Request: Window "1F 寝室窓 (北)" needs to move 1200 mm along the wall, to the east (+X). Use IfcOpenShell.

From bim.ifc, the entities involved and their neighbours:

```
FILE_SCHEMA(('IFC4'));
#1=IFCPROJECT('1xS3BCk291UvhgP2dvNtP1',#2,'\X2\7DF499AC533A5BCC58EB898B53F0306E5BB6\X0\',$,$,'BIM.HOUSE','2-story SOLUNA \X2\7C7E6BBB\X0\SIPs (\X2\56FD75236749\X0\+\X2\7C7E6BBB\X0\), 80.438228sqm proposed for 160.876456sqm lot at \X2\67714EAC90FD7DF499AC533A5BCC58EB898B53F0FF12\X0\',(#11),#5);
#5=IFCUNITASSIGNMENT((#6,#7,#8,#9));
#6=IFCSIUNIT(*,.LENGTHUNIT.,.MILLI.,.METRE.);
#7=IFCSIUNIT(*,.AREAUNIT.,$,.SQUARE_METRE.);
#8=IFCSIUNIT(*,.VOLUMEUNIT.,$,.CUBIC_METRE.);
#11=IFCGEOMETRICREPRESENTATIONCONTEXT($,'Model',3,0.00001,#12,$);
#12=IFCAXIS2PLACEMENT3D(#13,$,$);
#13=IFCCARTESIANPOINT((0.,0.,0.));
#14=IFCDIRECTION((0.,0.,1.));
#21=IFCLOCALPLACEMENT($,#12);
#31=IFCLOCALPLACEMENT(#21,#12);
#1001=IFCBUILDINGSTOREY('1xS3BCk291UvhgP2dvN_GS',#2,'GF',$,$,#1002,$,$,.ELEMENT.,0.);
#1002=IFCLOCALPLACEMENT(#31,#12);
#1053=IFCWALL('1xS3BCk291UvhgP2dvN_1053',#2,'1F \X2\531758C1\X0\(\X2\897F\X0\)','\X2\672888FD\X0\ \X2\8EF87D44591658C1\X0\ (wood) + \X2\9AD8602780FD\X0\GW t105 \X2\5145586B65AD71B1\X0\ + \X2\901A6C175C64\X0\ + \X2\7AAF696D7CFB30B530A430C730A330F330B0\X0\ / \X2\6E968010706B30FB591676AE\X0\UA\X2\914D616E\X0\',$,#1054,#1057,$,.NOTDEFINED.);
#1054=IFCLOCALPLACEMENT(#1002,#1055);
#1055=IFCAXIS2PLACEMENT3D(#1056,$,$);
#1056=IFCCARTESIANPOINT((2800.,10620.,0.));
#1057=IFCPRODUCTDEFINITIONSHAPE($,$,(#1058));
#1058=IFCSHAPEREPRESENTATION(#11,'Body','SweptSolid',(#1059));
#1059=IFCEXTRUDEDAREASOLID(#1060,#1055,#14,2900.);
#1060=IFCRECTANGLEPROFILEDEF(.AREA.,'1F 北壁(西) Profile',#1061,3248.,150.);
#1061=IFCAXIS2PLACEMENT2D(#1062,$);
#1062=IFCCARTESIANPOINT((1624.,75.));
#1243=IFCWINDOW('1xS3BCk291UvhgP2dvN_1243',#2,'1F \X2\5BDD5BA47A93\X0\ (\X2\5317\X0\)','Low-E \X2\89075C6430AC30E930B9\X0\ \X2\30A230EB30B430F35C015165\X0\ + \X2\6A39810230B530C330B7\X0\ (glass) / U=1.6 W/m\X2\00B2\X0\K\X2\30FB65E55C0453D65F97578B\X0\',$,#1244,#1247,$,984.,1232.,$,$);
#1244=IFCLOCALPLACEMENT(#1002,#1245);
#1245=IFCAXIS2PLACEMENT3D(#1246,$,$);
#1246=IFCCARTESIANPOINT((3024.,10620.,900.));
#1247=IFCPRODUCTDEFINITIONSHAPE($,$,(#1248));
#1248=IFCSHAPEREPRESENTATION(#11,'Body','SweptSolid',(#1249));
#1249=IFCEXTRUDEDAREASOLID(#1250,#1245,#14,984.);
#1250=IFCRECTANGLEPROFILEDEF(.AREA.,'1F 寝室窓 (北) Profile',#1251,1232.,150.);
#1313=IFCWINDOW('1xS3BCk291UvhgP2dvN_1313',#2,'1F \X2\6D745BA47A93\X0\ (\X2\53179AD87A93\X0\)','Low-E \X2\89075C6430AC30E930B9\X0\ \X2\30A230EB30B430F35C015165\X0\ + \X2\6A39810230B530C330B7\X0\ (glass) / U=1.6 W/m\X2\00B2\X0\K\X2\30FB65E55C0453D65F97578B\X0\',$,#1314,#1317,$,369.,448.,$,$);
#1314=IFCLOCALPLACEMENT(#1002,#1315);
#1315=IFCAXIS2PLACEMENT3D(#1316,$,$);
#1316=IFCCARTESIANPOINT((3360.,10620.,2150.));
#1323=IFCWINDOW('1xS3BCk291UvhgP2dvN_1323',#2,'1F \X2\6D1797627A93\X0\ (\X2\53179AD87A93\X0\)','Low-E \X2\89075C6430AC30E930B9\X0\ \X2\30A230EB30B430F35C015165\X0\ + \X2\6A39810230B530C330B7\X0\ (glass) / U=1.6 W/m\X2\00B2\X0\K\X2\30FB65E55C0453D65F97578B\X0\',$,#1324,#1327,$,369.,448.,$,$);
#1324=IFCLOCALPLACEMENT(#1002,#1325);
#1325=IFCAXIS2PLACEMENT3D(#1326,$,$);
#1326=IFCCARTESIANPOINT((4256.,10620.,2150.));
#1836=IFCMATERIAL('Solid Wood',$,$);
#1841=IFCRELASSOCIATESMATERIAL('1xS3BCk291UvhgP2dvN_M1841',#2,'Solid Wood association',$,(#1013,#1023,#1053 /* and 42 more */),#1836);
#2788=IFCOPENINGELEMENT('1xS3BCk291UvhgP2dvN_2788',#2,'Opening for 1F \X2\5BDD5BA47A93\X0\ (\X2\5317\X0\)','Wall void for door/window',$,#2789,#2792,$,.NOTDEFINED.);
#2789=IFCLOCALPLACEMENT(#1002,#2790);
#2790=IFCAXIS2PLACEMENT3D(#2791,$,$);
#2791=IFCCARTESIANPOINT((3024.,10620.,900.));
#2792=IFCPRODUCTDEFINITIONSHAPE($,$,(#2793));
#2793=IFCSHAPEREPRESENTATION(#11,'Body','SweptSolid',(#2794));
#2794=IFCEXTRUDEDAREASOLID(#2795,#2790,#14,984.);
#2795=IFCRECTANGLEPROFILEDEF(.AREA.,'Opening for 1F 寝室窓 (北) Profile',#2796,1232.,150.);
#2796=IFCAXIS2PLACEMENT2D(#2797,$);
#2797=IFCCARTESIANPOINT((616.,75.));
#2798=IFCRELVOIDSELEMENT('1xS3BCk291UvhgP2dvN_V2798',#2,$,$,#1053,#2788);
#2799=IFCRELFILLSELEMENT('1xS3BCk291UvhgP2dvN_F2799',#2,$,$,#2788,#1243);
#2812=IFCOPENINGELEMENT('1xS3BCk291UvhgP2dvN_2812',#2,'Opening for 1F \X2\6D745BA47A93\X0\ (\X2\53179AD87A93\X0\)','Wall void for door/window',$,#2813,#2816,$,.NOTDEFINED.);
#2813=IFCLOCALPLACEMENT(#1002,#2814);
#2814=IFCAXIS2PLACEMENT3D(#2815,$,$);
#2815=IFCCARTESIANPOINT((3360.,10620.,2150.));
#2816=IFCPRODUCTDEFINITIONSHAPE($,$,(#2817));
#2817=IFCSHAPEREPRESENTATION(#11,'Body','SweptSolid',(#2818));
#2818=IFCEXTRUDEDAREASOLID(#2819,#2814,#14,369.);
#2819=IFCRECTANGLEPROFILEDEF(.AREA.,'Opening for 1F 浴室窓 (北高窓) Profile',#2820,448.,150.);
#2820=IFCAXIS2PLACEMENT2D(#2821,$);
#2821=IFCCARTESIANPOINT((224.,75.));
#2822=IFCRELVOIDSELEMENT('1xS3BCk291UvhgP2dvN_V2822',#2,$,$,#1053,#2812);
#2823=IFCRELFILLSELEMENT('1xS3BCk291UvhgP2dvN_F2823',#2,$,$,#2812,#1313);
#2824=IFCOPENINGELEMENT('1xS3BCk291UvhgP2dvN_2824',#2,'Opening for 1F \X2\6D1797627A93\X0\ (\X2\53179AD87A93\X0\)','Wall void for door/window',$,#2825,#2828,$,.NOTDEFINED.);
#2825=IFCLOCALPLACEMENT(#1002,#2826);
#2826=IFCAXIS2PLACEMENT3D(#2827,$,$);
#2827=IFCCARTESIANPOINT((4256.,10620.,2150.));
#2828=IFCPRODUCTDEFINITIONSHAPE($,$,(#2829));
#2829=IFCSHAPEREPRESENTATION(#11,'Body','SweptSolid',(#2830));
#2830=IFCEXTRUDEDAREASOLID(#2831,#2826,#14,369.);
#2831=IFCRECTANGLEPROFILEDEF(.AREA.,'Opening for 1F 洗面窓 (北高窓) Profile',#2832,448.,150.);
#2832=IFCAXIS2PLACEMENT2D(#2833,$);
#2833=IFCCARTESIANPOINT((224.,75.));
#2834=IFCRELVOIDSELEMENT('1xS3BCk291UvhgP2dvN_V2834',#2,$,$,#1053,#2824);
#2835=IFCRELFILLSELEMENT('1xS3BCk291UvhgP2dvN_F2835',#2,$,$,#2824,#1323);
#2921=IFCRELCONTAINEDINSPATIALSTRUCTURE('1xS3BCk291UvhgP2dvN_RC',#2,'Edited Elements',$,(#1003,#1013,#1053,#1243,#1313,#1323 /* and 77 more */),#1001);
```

```python
import ifcopenshell
import ifcopenshell.api.geometry
import ifcopenshell.util.placement

model = ifcopenshell.open("bim.ifc")

window = model.by_id(1243)
opening = window.FillsVoids[0].RelatingOpeningElement
wall = opening.VoidsElements[0].RelatingBuildingElement

wall_matrix = ifcopenshell.util.placement.get_local_placement(wall.ObjectPlacement)
shift = wall_matrix[:3, 0] * 1200.0
before = ifcopenshell.util.placement.get_local_placement(window.ObjectPlacement)[:3, 3].copy()

# The window is not placed relative to its opening, so move both.
for product in (opening, window):
    matrix = ifcopenshell.util.placement.get_local_placement(product.ObjectPlacement)
    matrix[:3, 3] += shift
    ifcopenshell.api.geometry.edit_object_placement(model, product=product, matrix=matrix, is_si=False)

after = ifcopenshell.util.placement.get_local_placement(window.ObjectPlacement)[:3, 3]
print("window moved by", (after - before).round(3) + 0.0)

model.write("bim_edited.ifc")
```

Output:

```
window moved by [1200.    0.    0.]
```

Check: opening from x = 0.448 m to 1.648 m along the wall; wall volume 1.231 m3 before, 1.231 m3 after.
